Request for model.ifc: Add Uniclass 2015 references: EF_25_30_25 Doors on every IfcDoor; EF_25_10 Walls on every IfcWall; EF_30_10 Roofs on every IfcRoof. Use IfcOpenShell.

First a look at what the model holds.

```python
import ifcopenshell

model = ifcopenshell.open("model.ifc")
print(model.schema)
print("classifications:", [c.Name for c in model.by_type("IfcClassification")])
for ifc_class in ("IfcDoor", "IfcRoof", "IfcStair", "IfcWall", "IfcWindow"):
    print(ifc_class, len(model.by_type(ifc_class)))
```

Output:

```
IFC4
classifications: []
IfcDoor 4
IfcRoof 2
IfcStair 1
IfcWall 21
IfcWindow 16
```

```python
import ifcopenshell
import ifcopenshell.api.classification

model = ifcopenshell.open("model.ifc")

system = ifcopenshell.api.classification.add_classification(model, classification="Uniclass 2015")

codes = {
    "IfcDoor": ("EF_25_30_25", "Doors"),
    "IfcWall": ("EF_25_10", "Walls"),
    "IfcRoof": ("EF_30_10", "Roofs"),
}
for ifc_class, (code, name) in codes.items():
    products = model.by_type(ifc_class)
    ifcopenshell.api.classification.add_reference(
        model, products=products, classification=system, identification=code, name=name
    )
    print(code, len(products))

model.write("model_updated.ifc")
```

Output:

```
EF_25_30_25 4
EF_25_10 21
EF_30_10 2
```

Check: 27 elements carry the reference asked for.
